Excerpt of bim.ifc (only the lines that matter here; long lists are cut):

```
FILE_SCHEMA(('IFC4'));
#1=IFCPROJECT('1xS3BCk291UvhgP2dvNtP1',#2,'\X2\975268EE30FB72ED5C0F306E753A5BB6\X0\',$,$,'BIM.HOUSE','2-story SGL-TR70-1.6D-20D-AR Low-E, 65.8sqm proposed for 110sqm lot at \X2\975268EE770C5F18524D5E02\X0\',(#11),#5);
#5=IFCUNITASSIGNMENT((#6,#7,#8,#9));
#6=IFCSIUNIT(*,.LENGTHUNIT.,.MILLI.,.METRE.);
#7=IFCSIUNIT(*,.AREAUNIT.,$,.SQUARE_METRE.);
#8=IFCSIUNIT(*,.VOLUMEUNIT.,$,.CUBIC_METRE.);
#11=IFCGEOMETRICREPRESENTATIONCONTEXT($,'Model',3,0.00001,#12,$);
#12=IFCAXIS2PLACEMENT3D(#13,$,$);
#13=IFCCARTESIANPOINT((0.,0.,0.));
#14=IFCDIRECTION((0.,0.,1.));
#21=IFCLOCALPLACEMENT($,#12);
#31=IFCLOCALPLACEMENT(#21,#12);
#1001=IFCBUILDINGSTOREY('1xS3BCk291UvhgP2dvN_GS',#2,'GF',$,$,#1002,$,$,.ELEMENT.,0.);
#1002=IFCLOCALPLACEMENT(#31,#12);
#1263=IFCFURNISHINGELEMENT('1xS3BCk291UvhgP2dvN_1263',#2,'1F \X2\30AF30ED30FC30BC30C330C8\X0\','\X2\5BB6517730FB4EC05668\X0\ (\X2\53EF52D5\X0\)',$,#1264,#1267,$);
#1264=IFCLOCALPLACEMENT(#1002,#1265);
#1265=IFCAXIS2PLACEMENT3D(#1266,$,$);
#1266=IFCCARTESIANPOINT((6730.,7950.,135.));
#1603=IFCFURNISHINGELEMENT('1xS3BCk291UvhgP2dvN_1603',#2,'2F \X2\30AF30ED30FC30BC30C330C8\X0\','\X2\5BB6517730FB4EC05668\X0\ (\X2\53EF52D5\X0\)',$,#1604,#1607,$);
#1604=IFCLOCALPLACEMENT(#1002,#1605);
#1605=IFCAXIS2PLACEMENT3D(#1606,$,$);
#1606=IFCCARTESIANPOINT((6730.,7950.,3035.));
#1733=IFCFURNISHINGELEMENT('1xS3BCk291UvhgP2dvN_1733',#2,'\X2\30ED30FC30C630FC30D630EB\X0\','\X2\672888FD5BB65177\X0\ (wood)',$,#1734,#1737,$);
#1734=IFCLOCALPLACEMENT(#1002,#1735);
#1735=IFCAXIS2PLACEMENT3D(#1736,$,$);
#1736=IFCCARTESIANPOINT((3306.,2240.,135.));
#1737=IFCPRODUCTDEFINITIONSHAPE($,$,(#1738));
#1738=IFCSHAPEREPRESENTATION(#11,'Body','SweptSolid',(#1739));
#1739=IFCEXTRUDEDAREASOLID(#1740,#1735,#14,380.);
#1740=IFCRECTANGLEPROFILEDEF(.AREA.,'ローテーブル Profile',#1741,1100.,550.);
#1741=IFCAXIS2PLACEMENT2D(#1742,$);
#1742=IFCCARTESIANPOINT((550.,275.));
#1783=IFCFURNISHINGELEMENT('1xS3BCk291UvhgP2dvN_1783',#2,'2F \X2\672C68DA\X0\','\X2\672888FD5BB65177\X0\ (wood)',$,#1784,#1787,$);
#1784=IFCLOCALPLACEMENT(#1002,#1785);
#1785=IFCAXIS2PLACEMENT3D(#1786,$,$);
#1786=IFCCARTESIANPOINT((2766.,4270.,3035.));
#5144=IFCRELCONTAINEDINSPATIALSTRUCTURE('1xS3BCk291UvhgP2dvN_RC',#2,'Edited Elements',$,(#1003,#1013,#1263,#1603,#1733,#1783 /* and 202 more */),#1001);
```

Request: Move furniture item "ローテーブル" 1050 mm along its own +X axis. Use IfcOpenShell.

```python
import ifcopenshell
import ifcopenshell.api.geometry
import ifcopenshell.util.placement

model = ifcopenshell.open("bim.ifc")

item = model.by_id(1733)
matrix = ifcopenshell.util.placement.get_local_placement(item.ObjectPlacement)
matrix[:3, 3] += matrix[:3, 0] * 1050.0
ifcopenshell.api.geometry.edit_object_placement(model, product=item, matrix=matrix, is_si=False)

print(ifcopenshell.util.placement.get_local_placement(item.ObjectPlacement).round(3) + 0.0)

model.write("bim_v2.ifc")
```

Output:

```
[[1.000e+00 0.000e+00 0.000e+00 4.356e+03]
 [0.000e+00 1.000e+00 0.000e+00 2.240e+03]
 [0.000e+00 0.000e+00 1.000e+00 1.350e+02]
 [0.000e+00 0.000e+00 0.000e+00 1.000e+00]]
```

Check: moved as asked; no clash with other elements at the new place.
